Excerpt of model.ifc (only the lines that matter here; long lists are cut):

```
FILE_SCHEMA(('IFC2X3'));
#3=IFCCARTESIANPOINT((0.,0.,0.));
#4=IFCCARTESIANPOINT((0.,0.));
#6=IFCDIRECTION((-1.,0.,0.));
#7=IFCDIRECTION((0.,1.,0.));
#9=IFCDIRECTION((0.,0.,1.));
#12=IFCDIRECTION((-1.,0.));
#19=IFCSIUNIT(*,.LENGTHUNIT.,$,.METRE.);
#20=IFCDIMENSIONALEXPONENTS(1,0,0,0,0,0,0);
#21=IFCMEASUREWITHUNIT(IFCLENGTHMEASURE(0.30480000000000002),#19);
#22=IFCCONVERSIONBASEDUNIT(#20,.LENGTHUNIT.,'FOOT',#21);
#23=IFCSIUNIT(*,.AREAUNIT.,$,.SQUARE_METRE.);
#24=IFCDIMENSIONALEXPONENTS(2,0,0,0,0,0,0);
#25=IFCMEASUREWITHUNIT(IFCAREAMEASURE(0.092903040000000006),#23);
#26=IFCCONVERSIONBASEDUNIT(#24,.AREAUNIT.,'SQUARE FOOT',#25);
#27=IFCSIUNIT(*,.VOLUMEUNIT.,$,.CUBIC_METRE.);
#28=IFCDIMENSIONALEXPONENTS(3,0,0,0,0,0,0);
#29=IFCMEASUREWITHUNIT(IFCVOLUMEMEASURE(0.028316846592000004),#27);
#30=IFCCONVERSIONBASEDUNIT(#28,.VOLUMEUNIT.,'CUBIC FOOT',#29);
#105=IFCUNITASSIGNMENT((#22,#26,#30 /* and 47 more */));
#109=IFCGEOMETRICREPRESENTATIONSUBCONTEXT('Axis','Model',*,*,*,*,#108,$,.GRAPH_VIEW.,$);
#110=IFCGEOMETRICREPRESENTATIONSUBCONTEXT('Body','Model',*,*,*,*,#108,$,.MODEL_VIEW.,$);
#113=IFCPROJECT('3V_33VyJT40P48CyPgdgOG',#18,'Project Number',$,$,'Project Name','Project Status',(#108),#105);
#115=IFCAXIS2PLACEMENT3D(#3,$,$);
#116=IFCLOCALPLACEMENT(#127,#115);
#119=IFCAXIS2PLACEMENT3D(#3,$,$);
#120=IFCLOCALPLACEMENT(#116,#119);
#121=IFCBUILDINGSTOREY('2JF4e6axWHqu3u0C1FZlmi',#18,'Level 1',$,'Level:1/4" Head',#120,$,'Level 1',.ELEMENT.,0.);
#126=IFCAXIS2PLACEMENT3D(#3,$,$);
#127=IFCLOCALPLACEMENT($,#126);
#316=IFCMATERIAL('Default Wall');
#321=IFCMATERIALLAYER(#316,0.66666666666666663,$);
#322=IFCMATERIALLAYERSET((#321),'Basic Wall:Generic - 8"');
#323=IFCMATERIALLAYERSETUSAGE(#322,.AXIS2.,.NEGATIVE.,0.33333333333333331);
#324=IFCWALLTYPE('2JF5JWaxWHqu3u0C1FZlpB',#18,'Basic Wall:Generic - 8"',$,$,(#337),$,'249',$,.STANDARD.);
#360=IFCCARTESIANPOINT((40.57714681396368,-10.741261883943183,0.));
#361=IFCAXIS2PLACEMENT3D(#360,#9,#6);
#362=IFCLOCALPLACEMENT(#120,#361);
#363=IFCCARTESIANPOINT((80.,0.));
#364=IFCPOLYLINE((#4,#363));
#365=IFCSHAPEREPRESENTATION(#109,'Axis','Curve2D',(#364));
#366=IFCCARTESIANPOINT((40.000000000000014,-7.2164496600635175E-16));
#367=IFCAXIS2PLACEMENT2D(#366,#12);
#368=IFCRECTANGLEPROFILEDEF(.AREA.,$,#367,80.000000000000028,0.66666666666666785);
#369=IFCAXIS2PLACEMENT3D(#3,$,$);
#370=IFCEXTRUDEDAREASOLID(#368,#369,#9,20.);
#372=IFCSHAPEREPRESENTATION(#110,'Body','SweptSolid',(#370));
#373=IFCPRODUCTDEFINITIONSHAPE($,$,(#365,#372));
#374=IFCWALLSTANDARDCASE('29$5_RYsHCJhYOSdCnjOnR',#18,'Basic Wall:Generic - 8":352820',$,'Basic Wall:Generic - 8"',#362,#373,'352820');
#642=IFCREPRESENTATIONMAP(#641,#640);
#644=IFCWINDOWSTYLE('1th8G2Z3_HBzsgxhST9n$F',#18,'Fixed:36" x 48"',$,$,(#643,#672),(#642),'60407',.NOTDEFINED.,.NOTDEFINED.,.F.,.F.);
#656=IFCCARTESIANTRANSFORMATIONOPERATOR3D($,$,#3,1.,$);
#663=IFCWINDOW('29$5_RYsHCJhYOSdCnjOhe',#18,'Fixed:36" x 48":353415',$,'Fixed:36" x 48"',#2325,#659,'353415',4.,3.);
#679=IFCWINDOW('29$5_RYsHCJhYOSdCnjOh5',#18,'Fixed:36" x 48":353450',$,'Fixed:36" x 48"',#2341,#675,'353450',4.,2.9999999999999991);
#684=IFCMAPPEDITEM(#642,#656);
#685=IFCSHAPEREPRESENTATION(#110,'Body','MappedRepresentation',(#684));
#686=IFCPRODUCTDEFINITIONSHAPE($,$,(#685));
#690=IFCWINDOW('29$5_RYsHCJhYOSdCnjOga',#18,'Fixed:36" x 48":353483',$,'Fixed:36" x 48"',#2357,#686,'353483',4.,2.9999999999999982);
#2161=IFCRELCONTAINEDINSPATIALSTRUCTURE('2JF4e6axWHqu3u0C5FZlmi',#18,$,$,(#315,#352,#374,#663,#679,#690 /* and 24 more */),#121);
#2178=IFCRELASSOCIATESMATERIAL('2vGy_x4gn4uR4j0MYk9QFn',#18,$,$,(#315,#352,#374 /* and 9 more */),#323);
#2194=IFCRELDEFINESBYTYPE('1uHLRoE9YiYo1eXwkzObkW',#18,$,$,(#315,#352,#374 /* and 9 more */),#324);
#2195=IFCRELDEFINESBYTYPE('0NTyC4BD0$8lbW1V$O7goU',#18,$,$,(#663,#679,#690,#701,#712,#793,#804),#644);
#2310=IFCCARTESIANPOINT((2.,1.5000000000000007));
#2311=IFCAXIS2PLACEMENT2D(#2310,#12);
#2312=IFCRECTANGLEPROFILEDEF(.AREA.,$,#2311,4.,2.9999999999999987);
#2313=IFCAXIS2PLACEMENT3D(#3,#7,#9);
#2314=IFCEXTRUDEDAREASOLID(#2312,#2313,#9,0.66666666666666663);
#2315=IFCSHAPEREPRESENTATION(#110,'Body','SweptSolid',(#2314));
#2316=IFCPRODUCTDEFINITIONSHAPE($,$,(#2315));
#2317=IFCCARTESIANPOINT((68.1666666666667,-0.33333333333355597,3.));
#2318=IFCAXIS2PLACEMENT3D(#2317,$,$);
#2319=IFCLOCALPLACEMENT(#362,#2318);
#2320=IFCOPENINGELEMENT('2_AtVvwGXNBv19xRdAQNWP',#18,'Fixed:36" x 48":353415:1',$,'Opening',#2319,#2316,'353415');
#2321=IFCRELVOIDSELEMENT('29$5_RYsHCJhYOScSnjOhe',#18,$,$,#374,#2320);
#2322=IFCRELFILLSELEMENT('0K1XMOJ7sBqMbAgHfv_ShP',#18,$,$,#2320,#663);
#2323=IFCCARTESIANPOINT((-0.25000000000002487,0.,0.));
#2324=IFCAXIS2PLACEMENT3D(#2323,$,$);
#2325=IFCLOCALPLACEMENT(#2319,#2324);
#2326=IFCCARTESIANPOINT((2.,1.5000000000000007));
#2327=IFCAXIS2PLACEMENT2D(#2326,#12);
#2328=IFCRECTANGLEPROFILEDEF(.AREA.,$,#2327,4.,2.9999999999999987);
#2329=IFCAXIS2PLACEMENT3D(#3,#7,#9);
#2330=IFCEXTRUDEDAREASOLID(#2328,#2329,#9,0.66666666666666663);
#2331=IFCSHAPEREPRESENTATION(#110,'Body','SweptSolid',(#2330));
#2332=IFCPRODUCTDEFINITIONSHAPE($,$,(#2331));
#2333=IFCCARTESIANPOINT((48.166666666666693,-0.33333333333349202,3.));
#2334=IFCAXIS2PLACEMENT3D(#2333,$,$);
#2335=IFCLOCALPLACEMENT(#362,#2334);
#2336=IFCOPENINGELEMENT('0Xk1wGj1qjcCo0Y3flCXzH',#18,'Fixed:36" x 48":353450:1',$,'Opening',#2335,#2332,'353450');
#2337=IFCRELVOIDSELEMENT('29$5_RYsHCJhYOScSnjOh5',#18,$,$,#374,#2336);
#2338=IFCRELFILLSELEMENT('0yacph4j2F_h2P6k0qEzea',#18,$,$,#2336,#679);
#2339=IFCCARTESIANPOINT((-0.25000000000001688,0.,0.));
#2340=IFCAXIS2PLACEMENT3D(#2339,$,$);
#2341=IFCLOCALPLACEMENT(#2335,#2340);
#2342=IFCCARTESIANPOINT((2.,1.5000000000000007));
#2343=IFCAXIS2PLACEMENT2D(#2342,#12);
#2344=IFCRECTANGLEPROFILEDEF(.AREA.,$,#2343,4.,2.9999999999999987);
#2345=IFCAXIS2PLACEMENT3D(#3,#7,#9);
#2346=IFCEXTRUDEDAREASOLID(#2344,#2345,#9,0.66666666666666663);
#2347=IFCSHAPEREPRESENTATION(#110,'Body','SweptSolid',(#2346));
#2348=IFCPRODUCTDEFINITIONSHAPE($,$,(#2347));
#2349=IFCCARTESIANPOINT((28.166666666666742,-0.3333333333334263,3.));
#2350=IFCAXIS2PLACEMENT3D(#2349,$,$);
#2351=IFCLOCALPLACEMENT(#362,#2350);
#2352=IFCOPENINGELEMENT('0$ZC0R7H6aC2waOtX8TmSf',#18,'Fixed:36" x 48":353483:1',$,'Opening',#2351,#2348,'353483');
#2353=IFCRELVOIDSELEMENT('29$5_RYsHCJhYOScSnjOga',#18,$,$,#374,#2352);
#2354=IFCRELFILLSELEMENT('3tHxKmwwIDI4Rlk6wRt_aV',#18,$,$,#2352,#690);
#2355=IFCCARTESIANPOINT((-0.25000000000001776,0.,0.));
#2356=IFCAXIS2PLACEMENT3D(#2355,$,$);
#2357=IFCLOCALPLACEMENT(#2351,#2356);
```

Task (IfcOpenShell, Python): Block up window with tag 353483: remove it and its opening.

```python
import ifcopenshell
import ifcopenshell.api.feature
import ifcopenshell.api.root
import ifcopenshell.geom
import ifcopenshell.util.shape

model = ifcopenshell.open("model.ifc")
settings = ifcopenshell.geom.settings()


def volume(element):
    """Net volume in cubic metres, openings subtracted."""
    shape = ifcopenshell.geom.create_shape(settings, element)
    return ifcopenshell.util.shape.get_volume(shape.geometry)


window = model.by_id(690)
opening = window.FillsVoids[0].RelatingOpeningElement
wall = opening.VoidsElements[0].RelatingBuildingElement
before = volume(wall)

ifcopenshell.api.root.remove_product(model, product=window)
ifcopenshell.api.feature.remove_feature(model, feature=opening)

after = volume(wall)

print(f"wall volume {before:.3f} -> {after:.3f} m3")

model.write("model_updated.ifc")
```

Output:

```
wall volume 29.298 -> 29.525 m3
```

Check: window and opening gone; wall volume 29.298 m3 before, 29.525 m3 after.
